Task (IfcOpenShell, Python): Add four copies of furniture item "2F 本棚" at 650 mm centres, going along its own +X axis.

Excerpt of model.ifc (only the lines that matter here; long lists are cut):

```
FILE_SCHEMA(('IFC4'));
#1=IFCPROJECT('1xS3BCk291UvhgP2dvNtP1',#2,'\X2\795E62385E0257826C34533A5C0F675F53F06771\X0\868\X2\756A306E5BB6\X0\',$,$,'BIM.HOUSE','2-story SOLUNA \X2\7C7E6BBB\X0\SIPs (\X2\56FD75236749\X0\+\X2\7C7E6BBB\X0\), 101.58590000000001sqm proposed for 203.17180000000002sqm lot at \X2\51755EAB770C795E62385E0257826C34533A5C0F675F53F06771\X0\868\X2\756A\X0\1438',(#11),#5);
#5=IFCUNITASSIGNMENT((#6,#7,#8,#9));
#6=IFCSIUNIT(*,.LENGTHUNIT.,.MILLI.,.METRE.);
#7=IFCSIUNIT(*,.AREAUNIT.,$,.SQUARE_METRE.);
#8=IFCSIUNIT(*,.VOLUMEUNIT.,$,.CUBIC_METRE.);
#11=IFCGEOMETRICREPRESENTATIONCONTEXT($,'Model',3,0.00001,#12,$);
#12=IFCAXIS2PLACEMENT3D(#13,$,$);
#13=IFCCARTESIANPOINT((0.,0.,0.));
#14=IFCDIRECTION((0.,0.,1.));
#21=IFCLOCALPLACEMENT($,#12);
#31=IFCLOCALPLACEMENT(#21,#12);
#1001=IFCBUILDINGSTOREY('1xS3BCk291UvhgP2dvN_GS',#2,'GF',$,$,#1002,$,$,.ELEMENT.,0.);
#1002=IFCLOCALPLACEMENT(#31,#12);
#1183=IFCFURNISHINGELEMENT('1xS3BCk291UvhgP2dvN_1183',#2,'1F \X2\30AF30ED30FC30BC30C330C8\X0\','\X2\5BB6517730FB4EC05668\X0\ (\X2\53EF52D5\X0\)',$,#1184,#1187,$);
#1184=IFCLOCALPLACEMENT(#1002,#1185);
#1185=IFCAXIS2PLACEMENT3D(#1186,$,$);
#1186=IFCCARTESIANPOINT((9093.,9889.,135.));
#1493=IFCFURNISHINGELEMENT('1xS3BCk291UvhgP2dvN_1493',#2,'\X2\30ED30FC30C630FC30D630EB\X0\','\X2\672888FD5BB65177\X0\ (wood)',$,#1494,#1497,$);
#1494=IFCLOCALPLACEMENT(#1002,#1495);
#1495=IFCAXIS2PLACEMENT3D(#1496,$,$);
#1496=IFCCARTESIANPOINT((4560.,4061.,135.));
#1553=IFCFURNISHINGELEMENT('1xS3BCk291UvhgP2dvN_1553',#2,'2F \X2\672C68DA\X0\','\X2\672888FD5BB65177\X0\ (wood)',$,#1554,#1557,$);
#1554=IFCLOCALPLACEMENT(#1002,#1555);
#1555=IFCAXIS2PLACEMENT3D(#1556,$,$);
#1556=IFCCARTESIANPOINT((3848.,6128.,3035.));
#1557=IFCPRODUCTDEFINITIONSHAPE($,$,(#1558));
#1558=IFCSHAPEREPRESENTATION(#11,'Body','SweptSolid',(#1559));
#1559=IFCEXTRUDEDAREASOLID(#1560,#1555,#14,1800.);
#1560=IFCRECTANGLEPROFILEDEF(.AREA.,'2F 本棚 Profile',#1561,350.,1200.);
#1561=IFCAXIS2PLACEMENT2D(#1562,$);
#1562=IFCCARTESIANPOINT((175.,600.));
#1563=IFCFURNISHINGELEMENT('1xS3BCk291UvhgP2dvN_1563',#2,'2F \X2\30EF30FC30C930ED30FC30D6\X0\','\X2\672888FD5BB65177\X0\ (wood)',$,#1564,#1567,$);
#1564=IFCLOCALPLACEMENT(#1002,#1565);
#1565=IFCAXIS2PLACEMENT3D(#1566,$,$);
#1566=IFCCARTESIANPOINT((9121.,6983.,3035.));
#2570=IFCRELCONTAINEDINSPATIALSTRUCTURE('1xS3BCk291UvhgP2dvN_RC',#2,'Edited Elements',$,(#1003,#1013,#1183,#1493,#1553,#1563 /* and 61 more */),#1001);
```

```python
import ifcopenshell
import ifcopenshell.api.geometry
import ifcopenshell.api.root
import ifcopenshell.util.element
import ifcopenshell.util.placement

model = ifcopenshell.open("model.ifc")


def reuse_history(source, copy):
    """copy_class also copies each property set's owner history, people and application; keep the originals."""
    for rel in copy.IsDefinedBy:
        if rel.is_a("IfcRelDefinesByProperties") and (history := rel.RelatingPropertyDefinition.OwnerHistory):
            rel.RelatingPropertyDefinition.OwnerHistory = source.OwnerHistory
            ifcopenshell.util.element.remove_deep2(model, history)


source = model.by_id(1553)
base = ifcopenshell.util.placement.get_local_placement(source.ObjectPlacement)
step = base[:3, 0] * 650.0

for i in range(1, 5):
    copy = ifcopenshell.api.root.copy_class(model, product=source)
    copy.Representation = ifcopenshell.util.element.copy_deep(
        model, source.Representation, exclude=["IfcGeometricRepresentationContext", "IfcRepresentationMap"]
    )
    reuse_history(source, copy)
    matrix = base.copy()
    matrix[:3, 3] += i * step
    print("added at", matrix[:3, 3].round(3) + 0.0)
    ifcopenshell.api.geometry.edit_object_placement(model, product=copy, matrix=matrix, is_si=False)

model.write("model_rev.ifc")
```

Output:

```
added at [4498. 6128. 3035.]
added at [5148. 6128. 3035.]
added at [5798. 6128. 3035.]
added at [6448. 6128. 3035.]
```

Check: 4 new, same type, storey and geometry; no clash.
